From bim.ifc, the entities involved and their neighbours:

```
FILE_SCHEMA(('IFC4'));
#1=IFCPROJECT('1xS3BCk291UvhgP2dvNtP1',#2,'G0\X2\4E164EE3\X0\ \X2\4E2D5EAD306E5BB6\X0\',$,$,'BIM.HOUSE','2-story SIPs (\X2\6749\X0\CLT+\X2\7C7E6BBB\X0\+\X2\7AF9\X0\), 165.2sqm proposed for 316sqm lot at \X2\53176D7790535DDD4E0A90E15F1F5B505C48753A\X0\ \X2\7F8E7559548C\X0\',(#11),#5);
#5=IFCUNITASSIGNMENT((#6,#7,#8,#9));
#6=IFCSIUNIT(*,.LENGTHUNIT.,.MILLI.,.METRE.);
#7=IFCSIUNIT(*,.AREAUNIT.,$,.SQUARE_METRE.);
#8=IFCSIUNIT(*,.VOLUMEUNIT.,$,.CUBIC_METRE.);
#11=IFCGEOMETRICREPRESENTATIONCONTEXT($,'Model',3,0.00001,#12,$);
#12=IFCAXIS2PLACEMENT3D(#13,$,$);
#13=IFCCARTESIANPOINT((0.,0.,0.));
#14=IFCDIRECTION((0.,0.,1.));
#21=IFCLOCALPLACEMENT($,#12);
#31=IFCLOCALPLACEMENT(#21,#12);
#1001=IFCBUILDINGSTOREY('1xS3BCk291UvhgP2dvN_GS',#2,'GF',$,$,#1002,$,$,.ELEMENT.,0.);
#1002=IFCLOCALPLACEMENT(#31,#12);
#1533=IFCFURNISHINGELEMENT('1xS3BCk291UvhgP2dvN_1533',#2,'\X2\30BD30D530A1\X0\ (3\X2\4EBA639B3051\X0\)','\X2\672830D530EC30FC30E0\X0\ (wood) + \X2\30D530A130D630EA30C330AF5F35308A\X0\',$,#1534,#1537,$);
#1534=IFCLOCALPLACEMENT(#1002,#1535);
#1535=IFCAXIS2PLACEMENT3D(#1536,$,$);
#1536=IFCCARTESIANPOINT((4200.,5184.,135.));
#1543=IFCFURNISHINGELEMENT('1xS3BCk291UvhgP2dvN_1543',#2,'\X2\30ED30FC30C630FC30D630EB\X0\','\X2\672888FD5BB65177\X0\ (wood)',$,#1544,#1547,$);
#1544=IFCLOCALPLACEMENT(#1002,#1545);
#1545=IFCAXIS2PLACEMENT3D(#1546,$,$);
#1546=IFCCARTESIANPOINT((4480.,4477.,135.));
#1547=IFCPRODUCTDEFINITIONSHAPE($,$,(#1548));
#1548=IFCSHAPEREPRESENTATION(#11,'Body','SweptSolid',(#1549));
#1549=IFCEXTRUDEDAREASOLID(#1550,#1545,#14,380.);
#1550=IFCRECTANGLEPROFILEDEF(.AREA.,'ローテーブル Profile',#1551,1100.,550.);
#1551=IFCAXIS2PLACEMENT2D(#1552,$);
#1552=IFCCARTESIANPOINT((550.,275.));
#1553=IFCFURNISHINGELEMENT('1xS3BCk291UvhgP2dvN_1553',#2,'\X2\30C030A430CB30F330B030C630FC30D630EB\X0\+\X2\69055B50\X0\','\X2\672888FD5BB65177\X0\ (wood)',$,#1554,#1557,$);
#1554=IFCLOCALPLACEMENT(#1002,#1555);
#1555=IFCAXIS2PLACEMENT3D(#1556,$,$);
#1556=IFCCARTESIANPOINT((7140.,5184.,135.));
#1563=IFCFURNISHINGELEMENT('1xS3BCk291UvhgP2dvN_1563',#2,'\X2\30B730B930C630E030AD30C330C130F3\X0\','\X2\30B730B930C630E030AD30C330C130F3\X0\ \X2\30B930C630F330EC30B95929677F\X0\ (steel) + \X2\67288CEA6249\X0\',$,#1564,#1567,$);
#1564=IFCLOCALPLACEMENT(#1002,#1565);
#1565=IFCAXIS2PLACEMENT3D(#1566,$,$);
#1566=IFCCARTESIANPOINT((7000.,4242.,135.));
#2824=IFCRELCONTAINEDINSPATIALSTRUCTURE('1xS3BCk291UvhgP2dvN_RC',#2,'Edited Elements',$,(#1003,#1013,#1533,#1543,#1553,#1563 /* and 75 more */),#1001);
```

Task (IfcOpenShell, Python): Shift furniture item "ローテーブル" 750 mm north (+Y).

```python
import ifcopenshell
import ifcopenshell.api.geometry
import ifcopenshell.util.placement
import ifcopenshell.util.unit

model = ifcopenshell.open("bim.ifc")
unit_scale = ifcopenshell.util.unit.calculate_unit_scale(model)

item = model.by_guid("1xS3BCk291UvhgP2dvN_1543")
matrix = ifcopenshell.util.placement.get_local_placement(item.ObjectPlacement)
matrix[1, 3] += 0.75 / unit_scale
ifcopenshell.api.geometry.edit_object_placement(model, product=item, matrix=matrix, is_si=False)

print(ifcopenshell.util.placement.get_local_placement(item.ObjectPlacement).round(3) + 0.0)

model.write("bim_updated.ifc")
```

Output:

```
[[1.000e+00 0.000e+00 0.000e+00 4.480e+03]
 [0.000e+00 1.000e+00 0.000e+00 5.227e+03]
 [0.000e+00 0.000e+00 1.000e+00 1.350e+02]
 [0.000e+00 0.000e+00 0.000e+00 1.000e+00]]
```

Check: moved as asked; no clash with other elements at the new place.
